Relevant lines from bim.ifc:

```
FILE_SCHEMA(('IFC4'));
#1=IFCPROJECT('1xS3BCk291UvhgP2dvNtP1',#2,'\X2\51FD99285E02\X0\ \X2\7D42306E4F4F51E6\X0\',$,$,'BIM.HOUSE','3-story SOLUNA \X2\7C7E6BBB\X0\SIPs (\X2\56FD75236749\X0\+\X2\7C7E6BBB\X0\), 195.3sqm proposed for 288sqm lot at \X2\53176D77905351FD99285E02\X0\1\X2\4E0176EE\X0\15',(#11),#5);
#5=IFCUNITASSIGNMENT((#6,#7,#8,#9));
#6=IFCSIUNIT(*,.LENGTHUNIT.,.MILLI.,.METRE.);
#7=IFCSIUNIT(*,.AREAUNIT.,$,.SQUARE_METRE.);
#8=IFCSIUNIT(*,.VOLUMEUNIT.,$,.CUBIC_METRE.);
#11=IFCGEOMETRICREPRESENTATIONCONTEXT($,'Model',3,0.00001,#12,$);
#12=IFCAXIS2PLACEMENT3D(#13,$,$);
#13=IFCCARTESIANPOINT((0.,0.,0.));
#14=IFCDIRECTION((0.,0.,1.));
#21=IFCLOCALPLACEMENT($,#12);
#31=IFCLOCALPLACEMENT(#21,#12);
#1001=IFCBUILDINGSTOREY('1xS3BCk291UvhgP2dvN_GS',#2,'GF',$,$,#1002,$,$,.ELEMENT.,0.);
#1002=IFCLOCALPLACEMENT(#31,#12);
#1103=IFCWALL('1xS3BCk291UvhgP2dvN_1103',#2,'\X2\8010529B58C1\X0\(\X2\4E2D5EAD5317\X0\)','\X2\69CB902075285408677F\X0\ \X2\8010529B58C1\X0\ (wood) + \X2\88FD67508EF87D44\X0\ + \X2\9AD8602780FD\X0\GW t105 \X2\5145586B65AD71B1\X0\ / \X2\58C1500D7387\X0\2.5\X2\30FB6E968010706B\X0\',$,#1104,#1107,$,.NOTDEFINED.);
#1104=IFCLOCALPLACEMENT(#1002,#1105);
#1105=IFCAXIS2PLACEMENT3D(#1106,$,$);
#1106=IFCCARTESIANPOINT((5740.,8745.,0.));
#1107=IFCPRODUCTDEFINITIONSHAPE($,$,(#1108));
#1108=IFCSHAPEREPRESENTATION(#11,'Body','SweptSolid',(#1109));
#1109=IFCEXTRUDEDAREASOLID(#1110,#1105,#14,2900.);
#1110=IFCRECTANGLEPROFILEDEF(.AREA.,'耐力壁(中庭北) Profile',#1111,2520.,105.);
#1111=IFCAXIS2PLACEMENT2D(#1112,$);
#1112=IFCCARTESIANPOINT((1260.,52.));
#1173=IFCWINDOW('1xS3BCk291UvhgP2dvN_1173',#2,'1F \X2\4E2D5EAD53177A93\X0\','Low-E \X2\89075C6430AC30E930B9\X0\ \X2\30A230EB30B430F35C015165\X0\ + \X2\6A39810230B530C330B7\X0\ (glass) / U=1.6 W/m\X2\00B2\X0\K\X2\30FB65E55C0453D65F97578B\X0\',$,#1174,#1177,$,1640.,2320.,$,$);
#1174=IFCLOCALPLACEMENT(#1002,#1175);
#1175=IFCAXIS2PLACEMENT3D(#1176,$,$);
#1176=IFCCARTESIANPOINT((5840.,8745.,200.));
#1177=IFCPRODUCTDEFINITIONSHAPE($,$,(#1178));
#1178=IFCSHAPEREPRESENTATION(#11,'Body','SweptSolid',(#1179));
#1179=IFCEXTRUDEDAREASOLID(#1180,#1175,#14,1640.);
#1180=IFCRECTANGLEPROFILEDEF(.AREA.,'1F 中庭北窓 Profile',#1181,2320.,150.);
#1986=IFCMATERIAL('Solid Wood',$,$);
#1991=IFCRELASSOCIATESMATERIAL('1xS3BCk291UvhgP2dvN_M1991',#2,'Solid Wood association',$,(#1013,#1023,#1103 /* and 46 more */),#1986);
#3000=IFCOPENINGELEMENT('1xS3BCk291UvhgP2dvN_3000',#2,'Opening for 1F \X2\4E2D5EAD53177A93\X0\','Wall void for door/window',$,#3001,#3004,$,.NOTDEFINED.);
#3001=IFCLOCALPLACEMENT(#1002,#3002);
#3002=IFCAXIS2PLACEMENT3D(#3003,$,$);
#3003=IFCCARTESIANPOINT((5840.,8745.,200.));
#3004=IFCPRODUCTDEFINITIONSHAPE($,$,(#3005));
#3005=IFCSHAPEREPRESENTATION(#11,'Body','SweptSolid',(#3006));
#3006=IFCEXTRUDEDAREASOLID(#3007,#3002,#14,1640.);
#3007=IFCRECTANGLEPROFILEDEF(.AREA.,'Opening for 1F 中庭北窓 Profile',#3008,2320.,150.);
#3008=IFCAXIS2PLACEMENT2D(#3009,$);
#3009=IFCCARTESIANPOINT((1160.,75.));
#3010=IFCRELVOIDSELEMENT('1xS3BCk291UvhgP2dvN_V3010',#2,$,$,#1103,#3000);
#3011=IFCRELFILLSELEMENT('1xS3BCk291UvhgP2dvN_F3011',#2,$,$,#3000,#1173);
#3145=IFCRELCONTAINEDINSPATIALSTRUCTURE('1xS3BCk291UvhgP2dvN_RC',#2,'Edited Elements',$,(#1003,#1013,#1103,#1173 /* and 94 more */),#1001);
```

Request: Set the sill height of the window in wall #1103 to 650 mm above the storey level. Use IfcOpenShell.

```python
import numpy as np
import ifcopenshell
import ifcopenshell.api.geometry
import ifcopenshell.geom
import ifcopenshell.util.element
import ifcopenshell.util.placement
import ifcopenshell.util.shape
import ifcopenshell.util.unit

model = ifcopenshell.open("bim.ifc")
unit_scale = ifcopenshell.util.unit.calculate_unit_scale(model)

window = model.by_guid("1xS3BCk291UvhgP2dvN_1173")
opening = window.FillsVoids[0].RelatingOpeningElement
storey = ifcopenshell.util.element.get_container(window, ifc_class="IfcBuildingStorey")
level = ifcopenshell.util.placement.get_local_placement(storey.ObjectPlacement)[2, 3]

# The opening's origin need not be at the sill, so measure its lowest point.
shape = ifcopenshell.geom.create_shape(ifcopenshell.geom.settings(), opening)
bottom = ifcopenshell.util.shape.get_shape_bottom_elevation(shape, shape.geometry) / unit_scale
dz = level + 0.65 / unit_scale - bottom

shift = np.array([0.0, 0.0, dz])
# The window is not placed relative to its opening, so move both.
for product in (opening, window):
    matrix = ifcopenshell.util.placement.get_local_placement(product.ObjectPlacement)
    matrix[:3, 3] += shift
    ifcopenshell.api.geometry.edit_object_placement(model, product=product, matrix=matrix, is_si=False)

print(f"moved by {dz * unit_scale:+.3f} m")

model.write("bim_v2.ifc")
```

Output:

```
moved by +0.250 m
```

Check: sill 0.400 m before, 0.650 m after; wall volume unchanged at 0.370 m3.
